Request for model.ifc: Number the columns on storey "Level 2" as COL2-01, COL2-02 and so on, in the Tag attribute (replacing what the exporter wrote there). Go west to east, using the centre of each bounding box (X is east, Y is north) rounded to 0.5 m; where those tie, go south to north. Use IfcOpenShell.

First a look at what the model holds.

```python
import ifcopenshell
import ifcopenshell.util.element
import ifcopenshell.util.placement

model = ifcopenshell.open("model.ifc")
print(model.schema)
storey = next(s for s in model.by_type("IfcBuildingStorey") if s.Name == "Level 2")
columns = [e for e in ifcopenshell.util.element.get_decomposition(storey) if e.is_a("IfcColumn")]
for e in sorted(columns, key=lambda e: e.id()):
    origin = ifcopenshell.util.placement.get_local_placement(e.ObjectPlacement)[:3, 3]
    print(e.id(), e.Tag, e.Name, origin.round(2) + 0.0, sep=" | ")
```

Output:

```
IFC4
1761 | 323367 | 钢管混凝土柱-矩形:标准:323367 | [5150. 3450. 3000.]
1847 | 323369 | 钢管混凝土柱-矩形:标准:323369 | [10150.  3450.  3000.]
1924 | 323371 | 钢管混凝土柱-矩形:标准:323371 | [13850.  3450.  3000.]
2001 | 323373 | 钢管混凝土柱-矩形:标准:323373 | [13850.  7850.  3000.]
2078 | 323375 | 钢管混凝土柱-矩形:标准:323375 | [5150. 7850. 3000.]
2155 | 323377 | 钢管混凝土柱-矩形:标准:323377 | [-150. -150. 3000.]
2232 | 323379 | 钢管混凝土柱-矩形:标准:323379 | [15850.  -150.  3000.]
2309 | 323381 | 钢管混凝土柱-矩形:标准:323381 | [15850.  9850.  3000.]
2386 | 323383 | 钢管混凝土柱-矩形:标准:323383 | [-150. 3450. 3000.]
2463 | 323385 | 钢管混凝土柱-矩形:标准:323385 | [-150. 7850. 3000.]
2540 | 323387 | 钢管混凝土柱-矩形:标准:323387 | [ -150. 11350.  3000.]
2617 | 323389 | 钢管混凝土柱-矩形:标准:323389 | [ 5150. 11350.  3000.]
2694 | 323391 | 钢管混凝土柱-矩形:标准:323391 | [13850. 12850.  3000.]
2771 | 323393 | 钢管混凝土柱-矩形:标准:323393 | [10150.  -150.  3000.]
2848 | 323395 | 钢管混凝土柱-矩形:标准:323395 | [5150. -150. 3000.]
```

```python
import ifcopenshell
import ifcopenshell.geom
import ifcopenshell.util.element
import ifcopenshell.util.shape

model = ifcopenshell.open("model.ifc")
settings = ifcopenshell.geom.settings()
settings.set("use-world-coords", True)


def centre(element):
    shape = ifcopenshell.geom.create_shape(settings, element)
    return ifcopenshell.util.shape.get_bbox_centroid(shape.geometry)


storey = next(s for s in model.by_type("IfcBuildingStorey") if s.Name == "Level 2")
columns = [e for e in ifcopenshell.util.element.get_decomposition(storey) if e.is_a("IfcColumn")]

# Insertion points can sit at a corner or the storey origin, so sort by the geometry (in metres).
centres = {e: centre(e) for e in columns}
columns.sort(key=lambda e: (round(centres[e][0] / 0.5), centres[e][1]))

for i, e in enumerate(columns, start=1):
    number = f"COL2-{i:02d}"
    e.Tag = number
    print(e.id(), number)

model.write("model_edited.ifc")
```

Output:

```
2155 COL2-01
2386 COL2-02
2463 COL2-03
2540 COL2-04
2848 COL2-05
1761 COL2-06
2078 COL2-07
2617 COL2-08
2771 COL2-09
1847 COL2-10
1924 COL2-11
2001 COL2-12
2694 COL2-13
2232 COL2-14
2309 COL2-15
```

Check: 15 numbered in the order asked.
